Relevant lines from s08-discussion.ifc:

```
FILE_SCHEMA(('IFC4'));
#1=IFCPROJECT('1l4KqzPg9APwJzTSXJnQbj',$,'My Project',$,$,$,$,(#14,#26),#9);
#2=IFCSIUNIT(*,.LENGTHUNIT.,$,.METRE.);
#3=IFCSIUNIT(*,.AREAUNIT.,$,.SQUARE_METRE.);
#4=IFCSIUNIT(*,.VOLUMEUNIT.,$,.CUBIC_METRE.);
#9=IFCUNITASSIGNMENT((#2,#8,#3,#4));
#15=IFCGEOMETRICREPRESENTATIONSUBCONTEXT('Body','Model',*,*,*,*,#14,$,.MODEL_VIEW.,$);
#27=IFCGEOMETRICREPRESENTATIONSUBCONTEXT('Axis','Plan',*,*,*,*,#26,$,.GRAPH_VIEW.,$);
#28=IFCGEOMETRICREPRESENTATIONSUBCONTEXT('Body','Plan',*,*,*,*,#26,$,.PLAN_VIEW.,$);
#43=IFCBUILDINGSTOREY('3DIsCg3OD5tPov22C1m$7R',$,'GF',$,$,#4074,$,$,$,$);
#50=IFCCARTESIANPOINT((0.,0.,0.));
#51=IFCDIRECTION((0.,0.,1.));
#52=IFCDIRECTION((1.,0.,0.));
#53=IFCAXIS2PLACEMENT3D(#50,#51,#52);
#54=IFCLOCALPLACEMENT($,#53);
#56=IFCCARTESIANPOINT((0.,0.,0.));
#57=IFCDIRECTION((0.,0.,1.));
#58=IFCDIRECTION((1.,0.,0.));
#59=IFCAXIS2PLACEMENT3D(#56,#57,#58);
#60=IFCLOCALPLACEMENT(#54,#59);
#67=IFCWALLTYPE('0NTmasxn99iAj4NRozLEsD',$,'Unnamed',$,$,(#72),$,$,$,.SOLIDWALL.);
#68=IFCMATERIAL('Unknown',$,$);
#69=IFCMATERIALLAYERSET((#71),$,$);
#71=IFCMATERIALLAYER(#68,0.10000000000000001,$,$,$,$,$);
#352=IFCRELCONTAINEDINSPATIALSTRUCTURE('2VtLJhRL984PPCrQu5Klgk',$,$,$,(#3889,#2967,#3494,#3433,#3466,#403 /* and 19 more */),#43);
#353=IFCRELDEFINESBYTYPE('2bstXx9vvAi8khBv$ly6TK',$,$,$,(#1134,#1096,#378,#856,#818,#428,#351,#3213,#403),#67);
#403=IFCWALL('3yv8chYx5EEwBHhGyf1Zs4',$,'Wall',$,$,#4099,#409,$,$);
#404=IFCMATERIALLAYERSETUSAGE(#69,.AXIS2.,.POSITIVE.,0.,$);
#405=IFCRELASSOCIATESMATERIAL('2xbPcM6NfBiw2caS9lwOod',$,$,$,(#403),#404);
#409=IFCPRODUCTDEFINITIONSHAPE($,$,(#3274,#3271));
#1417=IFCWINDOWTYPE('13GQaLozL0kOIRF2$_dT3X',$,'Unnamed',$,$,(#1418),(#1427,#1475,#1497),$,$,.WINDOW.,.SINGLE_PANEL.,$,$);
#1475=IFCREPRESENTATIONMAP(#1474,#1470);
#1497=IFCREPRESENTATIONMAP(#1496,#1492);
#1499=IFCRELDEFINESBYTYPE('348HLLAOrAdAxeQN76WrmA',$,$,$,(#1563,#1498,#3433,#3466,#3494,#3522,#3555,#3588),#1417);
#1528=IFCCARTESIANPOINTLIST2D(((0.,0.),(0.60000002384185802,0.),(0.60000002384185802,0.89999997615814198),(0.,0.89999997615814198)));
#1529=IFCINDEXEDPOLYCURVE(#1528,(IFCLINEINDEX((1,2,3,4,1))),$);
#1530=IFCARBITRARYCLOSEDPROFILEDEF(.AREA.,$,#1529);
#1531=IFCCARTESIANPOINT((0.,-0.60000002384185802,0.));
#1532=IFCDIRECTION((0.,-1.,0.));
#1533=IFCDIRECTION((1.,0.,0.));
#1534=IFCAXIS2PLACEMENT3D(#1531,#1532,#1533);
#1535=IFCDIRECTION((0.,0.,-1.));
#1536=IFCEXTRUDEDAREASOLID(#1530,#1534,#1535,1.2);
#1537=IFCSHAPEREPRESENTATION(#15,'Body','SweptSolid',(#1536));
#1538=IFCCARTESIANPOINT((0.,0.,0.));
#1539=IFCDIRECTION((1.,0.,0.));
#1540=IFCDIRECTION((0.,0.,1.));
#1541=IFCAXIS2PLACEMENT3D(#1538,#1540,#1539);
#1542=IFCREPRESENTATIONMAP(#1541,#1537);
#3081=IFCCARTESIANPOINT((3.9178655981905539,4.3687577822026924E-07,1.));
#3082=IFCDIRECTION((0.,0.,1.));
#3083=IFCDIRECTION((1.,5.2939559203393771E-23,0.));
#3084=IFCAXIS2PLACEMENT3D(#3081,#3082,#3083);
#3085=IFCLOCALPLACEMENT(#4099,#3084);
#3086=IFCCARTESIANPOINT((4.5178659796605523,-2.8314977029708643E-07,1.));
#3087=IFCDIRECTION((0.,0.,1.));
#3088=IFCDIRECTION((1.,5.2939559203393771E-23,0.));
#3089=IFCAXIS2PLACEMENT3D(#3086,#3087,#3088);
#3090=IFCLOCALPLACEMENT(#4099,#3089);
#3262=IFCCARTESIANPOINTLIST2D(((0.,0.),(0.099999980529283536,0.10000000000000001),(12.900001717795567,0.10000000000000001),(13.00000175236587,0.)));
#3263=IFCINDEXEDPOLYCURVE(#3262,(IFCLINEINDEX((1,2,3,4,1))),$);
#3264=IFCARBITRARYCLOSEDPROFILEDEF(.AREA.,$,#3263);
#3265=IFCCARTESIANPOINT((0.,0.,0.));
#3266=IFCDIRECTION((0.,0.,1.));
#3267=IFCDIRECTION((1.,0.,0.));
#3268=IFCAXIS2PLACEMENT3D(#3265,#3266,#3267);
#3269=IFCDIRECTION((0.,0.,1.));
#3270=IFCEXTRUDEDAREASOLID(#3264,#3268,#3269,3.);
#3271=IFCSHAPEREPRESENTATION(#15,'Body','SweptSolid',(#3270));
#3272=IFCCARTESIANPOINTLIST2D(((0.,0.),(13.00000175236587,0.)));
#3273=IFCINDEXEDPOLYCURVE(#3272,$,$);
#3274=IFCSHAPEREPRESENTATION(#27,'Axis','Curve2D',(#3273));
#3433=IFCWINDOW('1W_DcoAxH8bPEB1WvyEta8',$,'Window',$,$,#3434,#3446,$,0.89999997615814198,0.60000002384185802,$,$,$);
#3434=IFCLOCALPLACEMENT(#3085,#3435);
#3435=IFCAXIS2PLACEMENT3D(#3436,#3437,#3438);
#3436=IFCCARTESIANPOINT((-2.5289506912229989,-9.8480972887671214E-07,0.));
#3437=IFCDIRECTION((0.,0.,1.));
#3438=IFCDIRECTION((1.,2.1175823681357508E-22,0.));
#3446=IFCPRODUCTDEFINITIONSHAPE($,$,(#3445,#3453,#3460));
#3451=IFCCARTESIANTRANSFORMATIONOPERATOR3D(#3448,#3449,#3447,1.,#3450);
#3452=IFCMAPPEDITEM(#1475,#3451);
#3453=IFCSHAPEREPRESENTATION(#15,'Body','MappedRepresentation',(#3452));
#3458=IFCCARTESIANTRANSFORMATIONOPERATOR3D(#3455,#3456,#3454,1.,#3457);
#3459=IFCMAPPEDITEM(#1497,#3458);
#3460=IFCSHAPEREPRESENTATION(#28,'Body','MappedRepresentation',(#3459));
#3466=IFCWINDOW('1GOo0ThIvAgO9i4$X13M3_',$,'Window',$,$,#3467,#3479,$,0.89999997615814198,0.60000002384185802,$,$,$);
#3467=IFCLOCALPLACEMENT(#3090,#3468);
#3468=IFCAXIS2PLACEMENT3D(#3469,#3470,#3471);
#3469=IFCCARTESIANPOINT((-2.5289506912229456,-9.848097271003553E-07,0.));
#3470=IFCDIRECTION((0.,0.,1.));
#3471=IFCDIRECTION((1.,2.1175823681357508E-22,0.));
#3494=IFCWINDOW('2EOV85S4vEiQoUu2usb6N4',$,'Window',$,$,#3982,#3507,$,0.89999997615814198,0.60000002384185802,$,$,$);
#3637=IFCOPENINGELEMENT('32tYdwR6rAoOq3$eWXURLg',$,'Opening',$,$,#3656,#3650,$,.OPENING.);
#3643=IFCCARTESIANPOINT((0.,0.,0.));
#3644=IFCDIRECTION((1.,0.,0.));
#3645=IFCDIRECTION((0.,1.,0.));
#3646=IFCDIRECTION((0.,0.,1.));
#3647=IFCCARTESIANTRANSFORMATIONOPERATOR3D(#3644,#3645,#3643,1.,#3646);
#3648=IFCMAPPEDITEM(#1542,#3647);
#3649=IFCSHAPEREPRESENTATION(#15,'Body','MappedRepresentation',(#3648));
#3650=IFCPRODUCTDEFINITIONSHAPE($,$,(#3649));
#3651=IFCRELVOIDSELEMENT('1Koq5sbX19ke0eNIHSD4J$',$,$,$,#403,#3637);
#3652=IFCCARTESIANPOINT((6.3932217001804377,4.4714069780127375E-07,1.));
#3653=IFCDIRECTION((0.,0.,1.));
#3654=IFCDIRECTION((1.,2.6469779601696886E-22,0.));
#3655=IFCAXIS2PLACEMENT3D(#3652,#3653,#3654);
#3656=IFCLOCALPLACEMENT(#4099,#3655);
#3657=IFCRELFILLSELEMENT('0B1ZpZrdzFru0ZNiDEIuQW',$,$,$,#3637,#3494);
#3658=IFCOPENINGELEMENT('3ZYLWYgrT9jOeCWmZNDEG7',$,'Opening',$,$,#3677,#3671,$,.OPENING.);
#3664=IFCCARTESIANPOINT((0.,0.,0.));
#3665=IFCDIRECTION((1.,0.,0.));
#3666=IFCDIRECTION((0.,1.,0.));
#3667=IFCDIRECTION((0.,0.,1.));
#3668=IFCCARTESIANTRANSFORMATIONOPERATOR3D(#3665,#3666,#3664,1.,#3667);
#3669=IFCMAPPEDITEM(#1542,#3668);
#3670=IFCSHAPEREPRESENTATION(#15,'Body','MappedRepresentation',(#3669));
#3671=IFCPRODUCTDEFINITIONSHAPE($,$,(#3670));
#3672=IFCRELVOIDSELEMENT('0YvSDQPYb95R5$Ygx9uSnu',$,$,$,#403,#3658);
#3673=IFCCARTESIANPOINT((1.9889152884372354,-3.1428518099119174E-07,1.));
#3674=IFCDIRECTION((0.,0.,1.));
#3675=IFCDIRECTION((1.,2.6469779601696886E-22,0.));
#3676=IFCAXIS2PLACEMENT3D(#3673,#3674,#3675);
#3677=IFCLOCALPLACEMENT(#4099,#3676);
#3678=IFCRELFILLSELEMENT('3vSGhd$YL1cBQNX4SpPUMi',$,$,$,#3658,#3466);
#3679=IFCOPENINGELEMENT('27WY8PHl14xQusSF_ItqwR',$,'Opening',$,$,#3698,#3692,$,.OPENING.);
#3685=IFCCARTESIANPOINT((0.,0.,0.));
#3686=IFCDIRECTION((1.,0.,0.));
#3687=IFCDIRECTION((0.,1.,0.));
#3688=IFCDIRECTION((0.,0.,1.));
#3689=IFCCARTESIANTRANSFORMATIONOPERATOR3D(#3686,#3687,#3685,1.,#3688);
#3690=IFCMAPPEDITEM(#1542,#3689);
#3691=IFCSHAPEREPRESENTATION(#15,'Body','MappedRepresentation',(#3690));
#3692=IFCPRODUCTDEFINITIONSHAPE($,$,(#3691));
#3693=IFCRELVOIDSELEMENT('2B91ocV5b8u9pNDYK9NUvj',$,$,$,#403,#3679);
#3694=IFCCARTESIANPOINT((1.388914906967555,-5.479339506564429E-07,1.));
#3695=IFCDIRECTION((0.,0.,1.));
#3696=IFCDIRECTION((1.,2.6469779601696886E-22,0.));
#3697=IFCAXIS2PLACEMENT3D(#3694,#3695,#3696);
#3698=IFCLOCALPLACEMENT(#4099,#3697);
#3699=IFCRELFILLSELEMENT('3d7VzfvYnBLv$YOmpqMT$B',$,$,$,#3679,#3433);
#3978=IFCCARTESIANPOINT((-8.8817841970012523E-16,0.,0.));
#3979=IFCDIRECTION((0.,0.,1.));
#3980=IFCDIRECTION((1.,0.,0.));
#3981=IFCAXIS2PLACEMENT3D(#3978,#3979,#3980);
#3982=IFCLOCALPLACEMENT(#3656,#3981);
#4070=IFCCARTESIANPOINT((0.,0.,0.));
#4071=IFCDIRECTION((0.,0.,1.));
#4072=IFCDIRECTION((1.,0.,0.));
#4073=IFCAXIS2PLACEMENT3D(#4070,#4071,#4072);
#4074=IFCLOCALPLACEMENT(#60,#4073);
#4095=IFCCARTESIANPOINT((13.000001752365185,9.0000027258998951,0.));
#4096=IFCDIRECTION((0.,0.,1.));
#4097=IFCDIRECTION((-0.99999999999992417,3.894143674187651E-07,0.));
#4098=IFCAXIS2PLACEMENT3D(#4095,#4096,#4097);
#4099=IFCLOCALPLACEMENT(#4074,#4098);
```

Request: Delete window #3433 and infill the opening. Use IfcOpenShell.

```python
import ifcopenshell
import ifcopenshell.api.feature
import ifcopenshell.api.root
import ifcopenshell.geom
import ifcopenshell.util.shape

model = ifcopenshell.open("s08-discussion.ifc")
settings = ifcopenshell.geom.settings()


def volume(element):
    """Net volume in cubic metres, openings subtracted."""
    shape = ifcopenshell.geom.create_shape(settings, element)
    return ifcopenshell.util.shape.get_volume(shape.geometry)


window = model.by_guid("1W_DcoAxH8bPEB1WvyEta8")
opening = window.FillsVoids[0].RelatingOpeningElement
wall = opening.VoidsElements[0].RelatingBuildingElement
before = volume(wall)

ifcopenshell.api.root.remove_product(model, product=window)
ifcopenshell.api.feature.remove_feature(model, feature=opening)

after = volume(wall)

print(f"wall volume {before:.3f} -> {after:.3f} m3")

model.write("s08-discussion_rev.ifc")
```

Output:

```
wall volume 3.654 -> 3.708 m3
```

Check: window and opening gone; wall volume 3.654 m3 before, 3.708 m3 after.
